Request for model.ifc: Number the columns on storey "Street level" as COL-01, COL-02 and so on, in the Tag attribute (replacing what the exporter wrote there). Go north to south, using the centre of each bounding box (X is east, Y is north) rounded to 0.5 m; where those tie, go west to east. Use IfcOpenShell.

First a look at what the model holds.

```python
import ifcopenshell
import ifcopenshell.util.element
import ifcopenshell.util.placement

model = ifcopenshell.open("model.ifc")
print(model.schema)
storey = next(s for s in model.by_type("IfcBuildingStorey") if s.Name == "Street level")
columns = [e for e in ifcopenshell.util.element.get_decomposition(storey) if e.is_a("IfcColumn")]
for e in sorted(columns, key=lambda e: e.id()):
    origin = ifcopenshell.util.placement.get_local_placement(e.ObjectPlacement)[:3, 3]
    print(e.id(), e.Tag, e.Name, origin.round(2) + 0.0, sep=" | ")
```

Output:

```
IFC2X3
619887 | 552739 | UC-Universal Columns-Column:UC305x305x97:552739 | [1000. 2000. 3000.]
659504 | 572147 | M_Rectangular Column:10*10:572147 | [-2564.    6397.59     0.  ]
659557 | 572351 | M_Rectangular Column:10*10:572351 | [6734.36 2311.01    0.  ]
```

```python
import ifcopenshell
import ifcopenshell.geom
import ifcopenshell.util.element
import ifcopenshell.util.shape

model = ifcopenshell.open("model.ifc")
settings = ifcopenshell.geom.settings()
settings.set("use-world-coords", True)


def centre(element):
    shape = ifcopenshell.geom.create_shape(settings, element)
    return ifcopenshell.util.shape.get_bbox_centroid(shape.geometry)


storey = next(s for s in model.by_type("IfcBuildingStorey") if s.Name == "Street level")
columns = [e for e in ifcopenshell.util.element.get_decomposition(storey) if e.is_a("IfcColumn")]

# Insertion points can sit at a corner or the storey origin, so sort by the geometry (in metres).
centres = {e: centre(e) for e in columns}
columns.sort(key=lambda e: (-round(centres[e][1] / 0.5), centres[e][0]))

for i, e in enumerate(columns, start=1):
    number = f"COL-{i:02d}"
    e.Tag = number
    print(e.id(), number)

model.write("model-out.ifc")
```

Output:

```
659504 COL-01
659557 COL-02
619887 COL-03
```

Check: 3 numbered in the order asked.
